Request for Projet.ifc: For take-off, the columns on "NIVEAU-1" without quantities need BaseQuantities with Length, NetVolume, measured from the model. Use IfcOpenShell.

First a look at what the model holds.

```python
import ifcopenshell
import ifcopenshell.util.element
import ifcopenshell.util.unit

model = ifcopenshell.open("Projet.ifc")
print(model.schema)
for unit_type in ("LENGTHUNIT", "AREAUNIT", "VOLUMEUNIT"):
    print(unit_type, ifcopenshell.util.unit.calculate_unit_scale(model, unit_type))
storey = next(s for s in model.by_type("IfcBuildingStorey") if s.Name == "NIVEAU-1")
columns = [e for e in ifcopenshell.util.element.get_decomposition(storey) if e.is_a("IfcColumn")]
for e in sorted(columns, key=lambda e: e.id()):
    print(e.id(), e.is_a(), e.Name, list(ifcopenshell.util.element.get_psets(e, qtos_only=True)), sep=" | ")
```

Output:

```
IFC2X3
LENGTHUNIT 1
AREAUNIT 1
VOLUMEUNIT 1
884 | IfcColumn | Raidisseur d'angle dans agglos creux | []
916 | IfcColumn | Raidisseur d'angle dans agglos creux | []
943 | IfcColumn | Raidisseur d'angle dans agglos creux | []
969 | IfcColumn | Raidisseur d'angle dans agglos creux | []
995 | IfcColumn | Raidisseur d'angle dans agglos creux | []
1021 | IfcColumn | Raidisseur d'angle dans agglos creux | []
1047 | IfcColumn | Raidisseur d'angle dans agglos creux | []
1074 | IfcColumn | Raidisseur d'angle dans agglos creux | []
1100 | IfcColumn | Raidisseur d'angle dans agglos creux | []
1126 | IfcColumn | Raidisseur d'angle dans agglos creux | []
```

```python
import ifcopenshell
import ifcopenshell.api.pset
import ifcopenshell.geom
import ifcopenshell.util.element
import ifcopenshell.util.shape
import ifcopenshell.util.unit

model = ifcopenshell.open("Projet.ifc")
unit_scale = ifcopenshell.util.unit.calculate_unit_scale(model)
volume_scale = ifcopenshell.util.unit.calculate_unit_scale(model, "VOLUMEUNIT")
settings = ifcopenshell.geom.settings()

storey = next(s for s in model.by_type("IfcBuildingStorey") if s.Name == "NIVEAU-1")
columns = [e for e in ifcopenshell.util.element.get_decomposition(storey) if e.is_a("IfcColumn")]

for e in sorted(columns, key=lambda e: e.id()):
    if ifcopenshell.util.element.get_psets(e, qtos_only=True, should_inherit=False):
        continue
    # Geometry comes back in metres, in the element's own axes.
    shape = ifcopenshell.geom.create_shape(settings, e)
    values = {
        "Length": ifcopenshell.util.shape.get_z(shape.geometry) / unit_scale,
        "NetVolume": ifcopenshell.util.shape.get_volume(shape.geometry) / volume_scale,
    }
    qto = ifcopenshell.api.pset.add_qto(model, product=e, name="BaseQuantities")
    ifcopenshell.api.pset.edit_qto(model, qto=qto, properties=values)
    print(e.id(), {k: round(v, 3) for k, v in values.items()})

model.write("Projet_updated.ifc")
```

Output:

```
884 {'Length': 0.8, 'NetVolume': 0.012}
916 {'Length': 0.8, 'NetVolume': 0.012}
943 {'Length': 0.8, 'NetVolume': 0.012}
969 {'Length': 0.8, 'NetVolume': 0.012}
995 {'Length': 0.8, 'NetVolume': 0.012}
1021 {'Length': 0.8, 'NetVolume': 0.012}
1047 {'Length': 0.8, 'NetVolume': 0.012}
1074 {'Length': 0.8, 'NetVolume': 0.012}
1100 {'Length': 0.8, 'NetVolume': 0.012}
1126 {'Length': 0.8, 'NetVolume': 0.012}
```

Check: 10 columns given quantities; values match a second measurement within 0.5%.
